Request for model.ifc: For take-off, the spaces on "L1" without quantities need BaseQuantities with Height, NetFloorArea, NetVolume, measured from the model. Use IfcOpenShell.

First a look at what the model holds.

```python
import ifcopenshell
import ifcopenshell.util.element
import ifcopenshell.util.unit

model = ifcopenshell.open("model.ifc")
print(model.schema)
for unit_type in ("LENGTHUNIT", "AREAUNIT", "VOLUMEUNIT"):
    print(unit_type, ifcopenshell.util.unit.calculate_unit_scale(model, unit_type))
storey = next(s for s in model.by_type("IfcBuildingStorey") if s.Name == "L1")
spaces = [e for e in ifcopenshell.util.element.get_decomposition(storey) if e.is_a("IfcSpace")]
for e in sorted(spaces, key=lambda e: e.id()):
    print(e.id(), e.is_a(), e.Name, list(ifcopenshell.util.element.get_psets(e, qtos_only=True)), sep=" | ")
```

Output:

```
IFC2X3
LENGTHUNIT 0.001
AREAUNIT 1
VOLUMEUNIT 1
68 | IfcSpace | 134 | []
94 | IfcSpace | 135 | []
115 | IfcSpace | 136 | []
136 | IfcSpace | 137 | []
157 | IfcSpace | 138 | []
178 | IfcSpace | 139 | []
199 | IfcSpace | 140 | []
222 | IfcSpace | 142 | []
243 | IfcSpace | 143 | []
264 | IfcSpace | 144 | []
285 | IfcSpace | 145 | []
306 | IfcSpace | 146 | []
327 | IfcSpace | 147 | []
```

```python
import ifcopenshell
import ifcopenshell.api.pset
import ifcopenshell.geom
import ifcopenshell.util.element
import ifcopenshell.util.shape
import ifcopenshell.util.unit

model = ifcopenshell.open("model.ifc")
unit_scale = ifcopenshell.util.unit.calculate_unit_scale(model)
area_scale = ifcopenshell.util.unit.calculate_unit_scale(model, "AREAUNIT")
volume_scale = ifcopenshell.util.unit.calculate_unit_scale(model, "VOLUMEUNIT")
settings = ifcopenshell.geom.settings()

storey = next(s for s in model.by_type("IfcBuildingStorey") if s.Name == "L1")
spaces = [e for e in ifcopenshell.util.element.get_decomposition(storey) if e.is_a("IfcSpace")]

for e in sorted(spaces, key=lambda e: e.id()):
    if ifcopenshell.util.element.get_psets(e, qtos_only=True, should_inherit=False):
        continue
    # Geometry comes back in metres, in the element's own axes.
    shape = ifcopenshell.geom.create_shape(settings, e)
    values = {
        "Height": ifcopenshell.util.shape.get_z(shape.geometry) / unit_scale,
        "NetFloorArea": ifcopenshell.util.shape.get_footprint_area(shape.geometry) / area_scale,
        "NetVolume": ifcopenshell.util.shape.get_volume(shape.geometry) / volume_scale,
    }
    qto = ifcopenshell.api.pset.add_qto(model, product=e, name="BaseQuantities")
    ifcopenshell.api.pset.edit_qto(model, qto=qto, properties=values)
    print(e.id(), {k: round(v, 3) for k, v in values.items()})

model.write("model_v2.ifc")
```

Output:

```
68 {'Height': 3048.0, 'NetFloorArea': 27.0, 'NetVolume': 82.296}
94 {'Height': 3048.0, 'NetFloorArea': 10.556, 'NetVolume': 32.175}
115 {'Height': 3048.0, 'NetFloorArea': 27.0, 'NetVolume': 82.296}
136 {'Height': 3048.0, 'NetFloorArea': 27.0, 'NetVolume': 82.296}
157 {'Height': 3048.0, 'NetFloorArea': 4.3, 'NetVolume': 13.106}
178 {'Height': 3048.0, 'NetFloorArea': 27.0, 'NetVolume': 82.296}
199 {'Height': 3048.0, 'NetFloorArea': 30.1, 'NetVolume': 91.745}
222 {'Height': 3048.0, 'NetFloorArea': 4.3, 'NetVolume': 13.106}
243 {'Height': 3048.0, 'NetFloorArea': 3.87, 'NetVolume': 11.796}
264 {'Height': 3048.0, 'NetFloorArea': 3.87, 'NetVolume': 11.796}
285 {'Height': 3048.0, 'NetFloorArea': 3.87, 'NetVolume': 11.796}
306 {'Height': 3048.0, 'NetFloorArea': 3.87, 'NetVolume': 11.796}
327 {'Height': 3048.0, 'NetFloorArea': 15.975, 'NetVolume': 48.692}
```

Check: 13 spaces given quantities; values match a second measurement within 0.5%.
